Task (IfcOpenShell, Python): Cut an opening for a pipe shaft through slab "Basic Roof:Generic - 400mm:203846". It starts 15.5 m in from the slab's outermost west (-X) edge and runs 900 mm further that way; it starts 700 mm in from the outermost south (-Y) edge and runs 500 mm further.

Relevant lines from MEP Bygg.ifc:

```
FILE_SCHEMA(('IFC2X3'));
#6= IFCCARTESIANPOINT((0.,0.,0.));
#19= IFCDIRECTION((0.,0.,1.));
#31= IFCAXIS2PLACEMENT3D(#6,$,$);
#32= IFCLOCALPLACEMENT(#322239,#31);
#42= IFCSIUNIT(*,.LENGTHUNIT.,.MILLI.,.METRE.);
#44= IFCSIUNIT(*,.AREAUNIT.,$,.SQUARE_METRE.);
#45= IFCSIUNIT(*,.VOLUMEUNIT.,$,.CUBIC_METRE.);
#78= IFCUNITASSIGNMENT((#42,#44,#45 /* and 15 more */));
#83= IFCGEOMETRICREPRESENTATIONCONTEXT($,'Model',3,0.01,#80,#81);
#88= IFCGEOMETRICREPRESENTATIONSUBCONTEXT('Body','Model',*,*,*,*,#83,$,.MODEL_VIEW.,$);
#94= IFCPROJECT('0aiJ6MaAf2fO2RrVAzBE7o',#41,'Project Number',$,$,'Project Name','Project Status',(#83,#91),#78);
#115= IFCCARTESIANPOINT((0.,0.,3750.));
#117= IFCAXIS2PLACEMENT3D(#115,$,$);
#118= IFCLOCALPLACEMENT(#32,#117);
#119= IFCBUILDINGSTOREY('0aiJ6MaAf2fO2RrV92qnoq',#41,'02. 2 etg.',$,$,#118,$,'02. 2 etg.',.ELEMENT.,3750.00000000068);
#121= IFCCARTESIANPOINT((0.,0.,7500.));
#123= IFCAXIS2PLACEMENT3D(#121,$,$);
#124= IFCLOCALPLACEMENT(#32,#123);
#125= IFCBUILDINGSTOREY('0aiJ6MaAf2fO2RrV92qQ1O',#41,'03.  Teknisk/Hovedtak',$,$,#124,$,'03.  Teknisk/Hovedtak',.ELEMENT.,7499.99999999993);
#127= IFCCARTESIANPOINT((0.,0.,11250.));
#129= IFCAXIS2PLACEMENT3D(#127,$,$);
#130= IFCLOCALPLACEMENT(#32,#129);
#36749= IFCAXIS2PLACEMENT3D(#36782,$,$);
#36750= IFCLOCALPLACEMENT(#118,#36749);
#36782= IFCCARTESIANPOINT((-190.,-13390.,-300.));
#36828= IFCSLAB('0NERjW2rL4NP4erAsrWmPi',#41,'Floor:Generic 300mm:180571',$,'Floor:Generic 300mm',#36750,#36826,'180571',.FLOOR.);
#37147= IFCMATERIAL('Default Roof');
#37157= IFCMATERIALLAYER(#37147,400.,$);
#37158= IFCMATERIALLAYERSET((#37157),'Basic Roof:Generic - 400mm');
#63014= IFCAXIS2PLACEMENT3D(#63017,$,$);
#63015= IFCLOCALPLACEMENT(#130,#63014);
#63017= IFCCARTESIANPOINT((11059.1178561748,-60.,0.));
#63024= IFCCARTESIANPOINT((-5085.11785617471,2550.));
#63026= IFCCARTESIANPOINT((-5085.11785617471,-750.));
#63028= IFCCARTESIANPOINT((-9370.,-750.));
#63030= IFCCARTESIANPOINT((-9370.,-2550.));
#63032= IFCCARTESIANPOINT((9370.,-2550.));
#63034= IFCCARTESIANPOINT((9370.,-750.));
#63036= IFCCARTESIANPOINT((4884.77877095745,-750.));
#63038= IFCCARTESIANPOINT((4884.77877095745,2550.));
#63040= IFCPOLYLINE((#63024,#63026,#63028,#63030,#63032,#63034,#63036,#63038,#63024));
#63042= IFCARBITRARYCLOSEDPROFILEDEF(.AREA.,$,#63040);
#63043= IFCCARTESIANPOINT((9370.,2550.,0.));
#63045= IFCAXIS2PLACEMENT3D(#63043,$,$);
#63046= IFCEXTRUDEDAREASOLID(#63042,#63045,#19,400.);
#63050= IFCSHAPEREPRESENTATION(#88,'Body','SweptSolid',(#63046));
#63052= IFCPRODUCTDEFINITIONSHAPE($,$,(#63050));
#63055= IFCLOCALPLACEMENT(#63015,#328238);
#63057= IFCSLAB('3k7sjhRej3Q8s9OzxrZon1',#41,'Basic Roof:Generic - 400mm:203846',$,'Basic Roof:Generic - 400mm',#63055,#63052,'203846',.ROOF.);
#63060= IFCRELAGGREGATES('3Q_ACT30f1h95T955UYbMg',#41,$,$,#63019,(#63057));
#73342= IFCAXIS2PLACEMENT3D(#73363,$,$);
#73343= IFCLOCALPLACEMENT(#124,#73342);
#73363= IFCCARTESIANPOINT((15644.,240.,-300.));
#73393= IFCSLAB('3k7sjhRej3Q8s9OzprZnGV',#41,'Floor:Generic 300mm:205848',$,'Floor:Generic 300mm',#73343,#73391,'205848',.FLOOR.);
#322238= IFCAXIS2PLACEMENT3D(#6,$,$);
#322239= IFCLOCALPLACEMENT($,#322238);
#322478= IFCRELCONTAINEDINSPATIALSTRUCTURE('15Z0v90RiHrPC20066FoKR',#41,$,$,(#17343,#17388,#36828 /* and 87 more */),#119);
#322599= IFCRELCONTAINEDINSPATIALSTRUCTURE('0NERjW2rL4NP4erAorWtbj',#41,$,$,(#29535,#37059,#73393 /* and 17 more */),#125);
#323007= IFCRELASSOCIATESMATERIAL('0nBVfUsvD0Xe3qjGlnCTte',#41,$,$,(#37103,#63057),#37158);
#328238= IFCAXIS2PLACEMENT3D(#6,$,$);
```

```python
import numpy as np
import ifcopenshell
import ifcopenshell.api.feature
import ifcopenshell.api.geometry
import ifcopenshell.api.root
import ifcopenshell.geom
import ifcopenshell.util.placement
import ifcopenshell.util.representation
import ifcopenshell.util.shape
import ifcopenshell.util.unit

model = ifcopenshell.open("MEP Bygg.ifc")
unit_scale = ifcopenshell.util.unit.calculate_unit_scale(model)
settings = ifcopenshell.geom.settings()


def volume(element):
    """Net volume in cubic metres, openings subtracted."""
    shape = ifcopenshell.geom.create_shape(settings, element)
    return ifcopenshell.util.shape.get_volume(shape.geometry)


slab = model.by_guid("3k7sjhRej3Q8s9OzxrZon1")
before = volume(slab)

# Extent in the slab's own axes, in metres. The edges named are its -X and -Y sides.
slab_shape = ifcopenshell.geom.create_shape(settings, slab)
vertices = ifcopenshell.util.shape.get_vertices(slab_shape.geometry)
x_min, y_min, bottom = vertices.min(axis=0)
top = vertices[:, 2].max()

opening = ifcopenshell.api.root.create_entity(model, ifc_class="IfcOpeningElement", name="Pipe shaft opening")
context = ifcopenshell.util.representation.get_context(model, "Model", "Body", "MODEL_VIEW")
width, depth = 0.9, 0.5
outline = [(0.0, 0.0), (width, 0.0), (width, depth), (0.0, depth), (0.0, 0.0)]
# Overshoot both faces by 50 mm so the cut is clean.
shape = ifcopenshell.api.geometry.add_slab_representation(
    model, context=context, depth=top - bottom + 0.1, polyline=outline
)
ifcopenshell.api.geometry.assign_representation(model, product=opening, representation=shape)

matrix = ifcopenshell.util.placement.get_local_placement(slab.ObjectPlacement)
matrix[:, 3] = matrix @ np.append(np.array([x_min + 15.5, y_min + 0.7, bottom - 0.05]) / unit_scale, 1.0)
ifcopenshell.api.geometry.edit_object_placement(model, product=opening, matrix=matrix, is_si=False)
ifcopenshell.api.feature.add_feature(model, feature=opening, element=slab)

after = volume(slab)

print(f"slab volume {before:.3f} -> {after:.3f} m3")

model.write("MEP Bygg-out.ifc")
```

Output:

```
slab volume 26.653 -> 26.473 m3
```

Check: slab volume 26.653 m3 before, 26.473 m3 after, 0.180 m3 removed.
